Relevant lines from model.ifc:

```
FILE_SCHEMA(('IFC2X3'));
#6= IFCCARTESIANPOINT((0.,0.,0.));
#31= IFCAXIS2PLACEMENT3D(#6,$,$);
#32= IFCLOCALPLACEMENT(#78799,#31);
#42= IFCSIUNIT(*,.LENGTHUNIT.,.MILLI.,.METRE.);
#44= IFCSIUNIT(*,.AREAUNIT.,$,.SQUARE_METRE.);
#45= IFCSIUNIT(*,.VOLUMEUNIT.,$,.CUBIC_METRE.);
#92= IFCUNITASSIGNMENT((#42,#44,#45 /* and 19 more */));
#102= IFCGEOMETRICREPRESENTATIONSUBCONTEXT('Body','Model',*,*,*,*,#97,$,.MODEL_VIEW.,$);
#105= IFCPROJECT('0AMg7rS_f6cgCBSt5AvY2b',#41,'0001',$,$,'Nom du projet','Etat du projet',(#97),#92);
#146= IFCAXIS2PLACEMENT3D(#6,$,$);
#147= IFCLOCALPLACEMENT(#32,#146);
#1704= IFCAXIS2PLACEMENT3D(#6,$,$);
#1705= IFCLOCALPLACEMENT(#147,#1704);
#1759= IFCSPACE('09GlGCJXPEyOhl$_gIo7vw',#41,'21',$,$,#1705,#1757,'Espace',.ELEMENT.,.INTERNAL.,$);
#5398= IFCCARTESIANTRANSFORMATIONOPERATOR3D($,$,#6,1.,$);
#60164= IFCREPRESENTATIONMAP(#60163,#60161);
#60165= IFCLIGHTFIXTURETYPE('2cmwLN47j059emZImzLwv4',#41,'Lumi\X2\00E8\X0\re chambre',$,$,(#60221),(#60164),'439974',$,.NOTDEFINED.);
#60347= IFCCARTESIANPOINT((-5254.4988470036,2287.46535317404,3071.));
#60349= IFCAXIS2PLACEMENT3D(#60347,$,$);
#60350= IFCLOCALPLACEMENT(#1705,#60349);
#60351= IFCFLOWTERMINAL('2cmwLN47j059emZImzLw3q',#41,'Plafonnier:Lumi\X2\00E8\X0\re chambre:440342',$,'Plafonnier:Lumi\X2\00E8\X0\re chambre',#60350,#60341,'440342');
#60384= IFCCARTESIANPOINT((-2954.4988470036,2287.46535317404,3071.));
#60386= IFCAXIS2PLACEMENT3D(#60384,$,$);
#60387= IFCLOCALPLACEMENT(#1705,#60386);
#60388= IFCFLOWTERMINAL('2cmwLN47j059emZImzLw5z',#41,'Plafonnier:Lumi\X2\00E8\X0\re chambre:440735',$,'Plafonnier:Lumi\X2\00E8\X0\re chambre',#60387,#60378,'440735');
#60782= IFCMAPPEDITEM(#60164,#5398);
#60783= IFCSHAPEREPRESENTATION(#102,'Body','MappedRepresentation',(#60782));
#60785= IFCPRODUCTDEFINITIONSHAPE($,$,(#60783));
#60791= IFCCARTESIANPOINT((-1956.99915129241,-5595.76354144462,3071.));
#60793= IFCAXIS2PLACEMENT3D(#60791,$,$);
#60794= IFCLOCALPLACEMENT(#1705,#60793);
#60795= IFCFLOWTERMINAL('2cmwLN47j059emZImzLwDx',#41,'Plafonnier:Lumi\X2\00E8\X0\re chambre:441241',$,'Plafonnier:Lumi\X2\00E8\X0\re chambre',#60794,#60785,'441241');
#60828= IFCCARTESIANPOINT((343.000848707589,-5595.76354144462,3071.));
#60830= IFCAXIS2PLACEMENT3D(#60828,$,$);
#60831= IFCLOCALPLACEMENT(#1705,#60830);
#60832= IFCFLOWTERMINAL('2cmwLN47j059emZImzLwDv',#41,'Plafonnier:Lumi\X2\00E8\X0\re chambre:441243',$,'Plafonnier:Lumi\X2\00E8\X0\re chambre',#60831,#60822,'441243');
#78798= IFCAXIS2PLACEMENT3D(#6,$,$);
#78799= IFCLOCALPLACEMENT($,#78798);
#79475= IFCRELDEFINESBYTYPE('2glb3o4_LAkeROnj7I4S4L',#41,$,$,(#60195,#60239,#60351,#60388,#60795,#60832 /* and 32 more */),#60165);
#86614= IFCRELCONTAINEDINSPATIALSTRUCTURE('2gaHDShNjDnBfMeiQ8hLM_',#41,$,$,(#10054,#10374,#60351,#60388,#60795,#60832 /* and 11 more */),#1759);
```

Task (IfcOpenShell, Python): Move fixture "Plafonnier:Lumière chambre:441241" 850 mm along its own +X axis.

```python
import ifcopenshell
import ifcopenshell.api.geometry
import ifcopenshell.util.placement
import ifcopenshell.util.unit

model = ifcopenshell.open("model.ifc")
unit_scale = ifcopenshell.util.unit.calculate_unit_scale(model)

item = model.by_id(60795)
matrix = ifcopenshell.util.placement.get_local_placement(item.ObjectPlacement)
matrix[:3, 3] += matrix[:3, 0] * 0.85 / unit_scale
ifcopenshell.api.geometry.edit_object_placement(model, product=item, matrix=matrix, is_si=False)

print(ifcopenshell.util.placement.get_local_placement(item.ObjectPlacement).round(3) + 0.0)

model.write("model_rev.ifc")
```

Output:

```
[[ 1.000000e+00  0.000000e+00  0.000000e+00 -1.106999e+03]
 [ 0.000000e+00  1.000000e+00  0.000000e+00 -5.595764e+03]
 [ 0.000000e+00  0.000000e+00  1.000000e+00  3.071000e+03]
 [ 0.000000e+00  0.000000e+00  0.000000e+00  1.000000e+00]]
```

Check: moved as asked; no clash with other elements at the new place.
